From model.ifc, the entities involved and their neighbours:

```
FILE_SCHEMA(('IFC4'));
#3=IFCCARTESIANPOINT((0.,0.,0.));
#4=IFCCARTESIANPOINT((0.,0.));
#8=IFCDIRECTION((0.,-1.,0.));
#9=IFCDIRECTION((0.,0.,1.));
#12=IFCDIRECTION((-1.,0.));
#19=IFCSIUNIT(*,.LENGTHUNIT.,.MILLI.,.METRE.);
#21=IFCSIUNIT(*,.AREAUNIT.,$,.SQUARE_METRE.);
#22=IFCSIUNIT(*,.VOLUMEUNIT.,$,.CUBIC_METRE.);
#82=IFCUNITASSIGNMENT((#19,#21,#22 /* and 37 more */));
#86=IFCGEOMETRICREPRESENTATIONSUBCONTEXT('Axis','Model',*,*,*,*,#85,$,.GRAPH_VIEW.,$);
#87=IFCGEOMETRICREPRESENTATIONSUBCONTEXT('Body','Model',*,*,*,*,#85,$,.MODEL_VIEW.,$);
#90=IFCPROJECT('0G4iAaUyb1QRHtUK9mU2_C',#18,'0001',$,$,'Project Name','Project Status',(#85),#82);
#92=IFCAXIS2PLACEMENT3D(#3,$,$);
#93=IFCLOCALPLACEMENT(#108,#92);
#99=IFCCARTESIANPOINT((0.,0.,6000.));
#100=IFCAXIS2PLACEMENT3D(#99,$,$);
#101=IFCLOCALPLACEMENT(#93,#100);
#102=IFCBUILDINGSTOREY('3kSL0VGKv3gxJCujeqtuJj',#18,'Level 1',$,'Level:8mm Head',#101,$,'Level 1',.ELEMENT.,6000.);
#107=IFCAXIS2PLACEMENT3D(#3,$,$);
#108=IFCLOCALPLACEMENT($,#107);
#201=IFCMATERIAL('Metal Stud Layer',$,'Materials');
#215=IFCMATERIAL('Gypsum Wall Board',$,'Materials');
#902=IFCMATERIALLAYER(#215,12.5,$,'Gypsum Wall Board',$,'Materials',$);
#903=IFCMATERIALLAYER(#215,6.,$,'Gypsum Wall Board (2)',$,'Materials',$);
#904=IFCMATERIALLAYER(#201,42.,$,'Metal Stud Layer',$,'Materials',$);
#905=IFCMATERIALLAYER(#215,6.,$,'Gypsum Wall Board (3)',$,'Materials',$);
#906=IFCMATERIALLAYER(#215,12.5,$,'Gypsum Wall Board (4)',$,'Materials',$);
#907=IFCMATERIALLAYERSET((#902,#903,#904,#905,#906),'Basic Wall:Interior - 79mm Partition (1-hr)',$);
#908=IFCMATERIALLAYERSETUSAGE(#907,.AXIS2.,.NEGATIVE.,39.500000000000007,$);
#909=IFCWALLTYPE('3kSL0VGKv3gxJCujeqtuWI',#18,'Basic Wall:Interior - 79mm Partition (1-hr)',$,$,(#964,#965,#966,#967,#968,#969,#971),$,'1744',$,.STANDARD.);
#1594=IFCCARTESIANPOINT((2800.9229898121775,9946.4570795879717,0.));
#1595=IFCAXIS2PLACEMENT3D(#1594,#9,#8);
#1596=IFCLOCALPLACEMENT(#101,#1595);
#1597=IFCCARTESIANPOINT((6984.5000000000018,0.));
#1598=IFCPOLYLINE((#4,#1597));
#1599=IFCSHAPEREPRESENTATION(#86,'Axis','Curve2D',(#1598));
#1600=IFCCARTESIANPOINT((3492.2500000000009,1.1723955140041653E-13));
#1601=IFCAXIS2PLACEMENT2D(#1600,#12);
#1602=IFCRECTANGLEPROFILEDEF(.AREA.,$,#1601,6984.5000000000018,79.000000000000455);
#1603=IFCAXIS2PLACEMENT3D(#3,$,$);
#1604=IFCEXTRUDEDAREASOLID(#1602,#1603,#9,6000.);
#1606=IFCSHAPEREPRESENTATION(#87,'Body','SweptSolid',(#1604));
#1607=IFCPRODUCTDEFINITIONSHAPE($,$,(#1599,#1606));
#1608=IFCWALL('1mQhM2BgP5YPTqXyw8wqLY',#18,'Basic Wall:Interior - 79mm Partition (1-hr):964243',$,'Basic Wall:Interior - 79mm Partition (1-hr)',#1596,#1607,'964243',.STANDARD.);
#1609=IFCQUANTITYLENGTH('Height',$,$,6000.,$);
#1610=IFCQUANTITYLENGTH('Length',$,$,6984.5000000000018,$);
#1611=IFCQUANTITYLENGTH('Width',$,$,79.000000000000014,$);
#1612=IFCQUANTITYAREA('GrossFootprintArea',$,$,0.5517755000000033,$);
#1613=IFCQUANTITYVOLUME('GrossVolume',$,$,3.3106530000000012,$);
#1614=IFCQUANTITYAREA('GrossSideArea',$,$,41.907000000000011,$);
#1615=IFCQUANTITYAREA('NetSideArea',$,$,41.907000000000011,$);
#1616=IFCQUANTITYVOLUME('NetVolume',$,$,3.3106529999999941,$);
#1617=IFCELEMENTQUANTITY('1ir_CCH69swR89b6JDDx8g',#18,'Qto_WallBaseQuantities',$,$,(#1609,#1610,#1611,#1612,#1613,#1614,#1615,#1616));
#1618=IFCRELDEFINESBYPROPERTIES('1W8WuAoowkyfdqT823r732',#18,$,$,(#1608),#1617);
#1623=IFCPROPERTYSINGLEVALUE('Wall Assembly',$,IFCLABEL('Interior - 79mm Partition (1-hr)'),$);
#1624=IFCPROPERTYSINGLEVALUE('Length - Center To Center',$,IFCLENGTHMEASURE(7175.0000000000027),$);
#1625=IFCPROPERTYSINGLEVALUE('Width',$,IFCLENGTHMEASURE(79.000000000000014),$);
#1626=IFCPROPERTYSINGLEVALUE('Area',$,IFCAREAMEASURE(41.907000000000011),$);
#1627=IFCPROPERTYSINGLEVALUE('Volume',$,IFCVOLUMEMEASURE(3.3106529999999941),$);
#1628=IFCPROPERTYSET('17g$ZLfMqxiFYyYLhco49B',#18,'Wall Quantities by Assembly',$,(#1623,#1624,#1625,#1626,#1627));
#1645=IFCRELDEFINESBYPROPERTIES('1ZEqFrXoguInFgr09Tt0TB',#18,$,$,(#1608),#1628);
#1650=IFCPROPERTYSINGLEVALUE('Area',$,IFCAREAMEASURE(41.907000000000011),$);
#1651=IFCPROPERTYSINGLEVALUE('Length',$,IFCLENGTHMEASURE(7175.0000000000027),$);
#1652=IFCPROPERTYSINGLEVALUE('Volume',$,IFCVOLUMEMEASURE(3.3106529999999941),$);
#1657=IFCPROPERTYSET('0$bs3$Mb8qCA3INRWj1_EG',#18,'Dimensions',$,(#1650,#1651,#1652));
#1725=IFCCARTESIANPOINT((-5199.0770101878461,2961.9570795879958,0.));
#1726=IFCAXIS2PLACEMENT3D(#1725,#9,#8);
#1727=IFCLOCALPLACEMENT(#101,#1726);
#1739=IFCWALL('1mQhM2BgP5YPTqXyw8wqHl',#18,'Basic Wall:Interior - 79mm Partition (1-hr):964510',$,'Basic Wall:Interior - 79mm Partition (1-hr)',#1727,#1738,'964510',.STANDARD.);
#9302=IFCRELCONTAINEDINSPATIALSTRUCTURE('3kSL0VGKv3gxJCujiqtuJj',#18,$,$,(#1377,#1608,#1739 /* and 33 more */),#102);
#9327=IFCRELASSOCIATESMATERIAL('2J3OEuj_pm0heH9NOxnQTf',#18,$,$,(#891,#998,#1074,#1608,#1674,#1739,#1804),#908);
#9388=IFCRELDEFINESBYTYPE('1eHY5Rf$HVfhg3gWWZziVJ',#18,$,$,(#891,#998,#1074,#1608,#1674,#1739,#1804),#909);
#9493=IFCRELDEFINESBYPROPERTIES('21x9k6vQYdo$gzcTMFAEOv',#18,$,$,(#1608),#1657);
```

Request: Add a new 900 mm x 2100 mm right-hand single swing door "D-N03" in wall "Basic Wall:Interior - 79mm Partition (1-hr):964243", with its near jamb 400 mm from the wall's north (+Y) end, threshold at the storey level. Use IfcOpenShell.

```python
import numpy as np
import ifcopenshell
import ifcopenshell.api.feature
import ifcopenshell.api.geometry
import ifcopenshell.api.pset
import ifcopenshell.api.root
import ifcopenshell.api.spatial
import ifcopenshell.geom
import ifcopenshell.util.element
import ifcopenshell.util.placement
import ifcopenshell.util.representation
import ifcopenshell.util.shape
import ifcopenshell.util.unit

model = ifcopenshell.open("model.ifc")
unit_scale = ifcopenshell.util.unit.calculate_unit_scale(model)
area_scale = ifcopenshell.util.unit.calculate_unit_scale(model, "AREAUNIT")
volume_scale = ifcopenshell.util.unit.calculate_unit_scale(model, "VOLUMEUNIT")
settings = ifcopenshell.geom.settings()


def volume(element):
    """Net volume in cubic metres, openings subtracted."""
    shape = ifcopenshell.geom.create_shape(settings, element)
    return ifcopenshell.util.shape.get_volume(shape.geometry)


wall = model.by_guid("1mQhM2BgP5YPTqXyw8wqLY")
storey = ifcopenshell.util.element.get_container(wall, ifc_class="IfcBuildingStorey")
context = ifcopenshell.util.representation.get_context(model, "Model", "Body", "MODEL_VIEW")
before = volume(wall)

width, height, from_end, sill = 0.9, 2.1, 0.4, 0.0  # metres

# The wall runs along its own X axis, and the end named is its -X end.
wall_shape = ifcopenshell.geom.create_shape(settings, wall)
x, y, z = ifcopenshell.util.shape.get_vertices(wall_shape.geometry).T
start = x.min() + from_end
face, thickness = float(y.min()), float(y.max() - y.min())
wall_matrix = ifcopenshell.util.placement.get_local_placement(wall.ObjectPlacement)
level = ifcopenshell.util.placement.get_local_placement(storey.ObjectPlacement)[2, 3]


def in_wall(x, y):
    """Placement at x, y metres in the wall's axes, at sill height."""
    matrix = wall_matrix.copy()
    matrix[:, 3] = wall_matrix @ np.array([x / unit_scale, y / unit_scale, 0.0, 1.0])
    matrix[2, 3] = level + sill / unit_scale
    return matrix


# Opening: a box that overshoots both wall faces by 50 mm.
opening = ifcopenshell.api.root.create_entity(model, ifc_class="IfcOpeningElement", predefined_type="OPENING")
box = ifcopenshell.api.geometry.add_wall_representation(
    model, context=context, length=width, height=height, thickness=thickness + 0.1
)
ifcopenshell.api.geometry.assign_representation(model, product=opening, representation=box)
ifcopenshell.api.geometry.edit_object_placement(model, product=opening, matrix=in_wall(start, face - 0.05), is_si=False)
ifcopenshell.api.feature.add_feature(model, feature=opening, element=wall)

door = ifcopenshell.api.root.create_entity(model, ifc_class="IfcDoor", name="D-N03", predefined_type="DOOR")
door.OverallWidth, door.OverallHeight = width / unit_scale, height / unit_scale
door.OperationType = "SINGLE_SWING_RIGHT"
body = ifcopenshell.api.geometry.add_door_representation(
    model,
    context=context,
    overall_width=door.OverallWidth,
    overall_height=door.OverallHeight,
    operation_type="SINGLE_SWING_RIGHT",
    lining_properties={"LiningDepth": thickness / unit_scale, "ThresholdDepth": thickness / unit_scale},
)
ifcopenshell.api.geometry.assign_representation(model, product=door, representation=body)
ifcopenshell.api.spatial.assign_container(model, products=[door], relating_structure=storey)
ifcopenshell.api.feature.add_filling(model, opening=opening, element=door)

# The lining spans the wall, so the door starts at the wall face.
ifcopenshell.api.geometry.edit_object_placement(model, product=door, matrix=in_wall(start, face), is_si=False)

after = volume(wall)

# Update the wall's stored quantities.
qto = model.by_id(ifcopenshell.util.element.get_pset(wall, "Qto_WallBaseQuantities", should_inherit=False)["id"])
ifcopenshell.api.pset.edit_qto(model, qto=qto, properties={
    "NetSideArea": after / thickness / area_scale,
    "NetVolume": after / volume_scale,
})
pset = model.by_id(ifcopenshell.util.element.get_pset(wall, "Wall Quantities by Assembly", should_inherit=False)["id"])
ifcopenshell.api.pset.edit_pset(model, pset=pset, properties={
    "Area": model.create_entity("IfcAreaMeasure", after / thickness / area_scale),
    "Volume": model.create_entity("IfcVolumeMeasure", after / volume_scale),
})
pset = model.by_id(ifcopenshell.util.element.get_pset(wall, "Dimensions", should_inherit=False)["id"])
ifcopenshell.api.pset.edit_pset(model, pset=pset, properties={
    "Area": model.create_entity("IfcAreaMeasure", after / thickness / area_scale),
    "Volume": model.create_entity("IfcVolumeMeasure", after / volume_scale),
})

print(f"wall volume {before:.3f} -> {after:.3f} m3")

model.write("model_rev.ifc")
```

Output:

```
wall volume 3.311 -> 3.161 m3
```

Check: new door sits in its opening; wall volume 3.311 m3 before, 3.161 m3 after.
